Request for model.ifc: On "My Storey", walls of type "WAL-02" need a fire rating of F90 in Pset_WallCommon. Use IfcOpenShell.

First a look at what the model holds.

```python
import ifcopenshell
import ifcopenshell.util.element

model = ifcopenshell.open("model.ifc")
print(model.schema)
storey = next(s for s in model.by_type("IfcBuildingStorey") if s.Name == "My Storey")
walls = [e for e in ifcopenshell.util.element.get_decomposition(storey) if e.is_a("IfcWall")]
seen = {}
for e in walls:
    element_type = ifcopenshell.util.element.get_type(e)
    key = (element_type.Name if element_type != e and element_type else None, ifcopenshell.util.element.get_pset(e, "Pset_WallCommon", "FireRating"))
    seen[key] = seen.get(key, 0) + 1
for (name, value), count in sorted(seen.items(), key=str):
    print(count, "x", name, "|", value)
```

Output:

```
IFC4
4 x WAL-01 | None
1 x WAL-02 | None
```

```python
import ifcopenshell
import ifcopenshell.api.pset
import ifcopenshell.util.element

model = ifcopenshell.open("model.ifc")

storey = next(s for s in model.by_type("IfcBuildingStorey") if s.Name == "My Storey")
walls = [e for e in ifcopenshell.util.element.get_decomposition(storey) if e.is_a("IfcWall")]

count = 0
for e in walls:
    element_type = ifcopenshell.util.element.get_type(e)
    if element_type in (None, e) or element_type.Name != "WAL-02":
        continue
    # add_pset returns the element's existing set when there is one.
    pset = ifcopenshell.api.pset.add_pset(model, product=e, name="Pset_WallCommon")
    ifcopenshell.api.pset.edit_pset(model, pset=pset, properties={"FireRating": "F90"})
    count += 1

print(count, "walls updated")

model.write("model_v2.ifc")
```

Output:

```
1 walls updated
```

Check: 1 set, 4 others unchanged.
